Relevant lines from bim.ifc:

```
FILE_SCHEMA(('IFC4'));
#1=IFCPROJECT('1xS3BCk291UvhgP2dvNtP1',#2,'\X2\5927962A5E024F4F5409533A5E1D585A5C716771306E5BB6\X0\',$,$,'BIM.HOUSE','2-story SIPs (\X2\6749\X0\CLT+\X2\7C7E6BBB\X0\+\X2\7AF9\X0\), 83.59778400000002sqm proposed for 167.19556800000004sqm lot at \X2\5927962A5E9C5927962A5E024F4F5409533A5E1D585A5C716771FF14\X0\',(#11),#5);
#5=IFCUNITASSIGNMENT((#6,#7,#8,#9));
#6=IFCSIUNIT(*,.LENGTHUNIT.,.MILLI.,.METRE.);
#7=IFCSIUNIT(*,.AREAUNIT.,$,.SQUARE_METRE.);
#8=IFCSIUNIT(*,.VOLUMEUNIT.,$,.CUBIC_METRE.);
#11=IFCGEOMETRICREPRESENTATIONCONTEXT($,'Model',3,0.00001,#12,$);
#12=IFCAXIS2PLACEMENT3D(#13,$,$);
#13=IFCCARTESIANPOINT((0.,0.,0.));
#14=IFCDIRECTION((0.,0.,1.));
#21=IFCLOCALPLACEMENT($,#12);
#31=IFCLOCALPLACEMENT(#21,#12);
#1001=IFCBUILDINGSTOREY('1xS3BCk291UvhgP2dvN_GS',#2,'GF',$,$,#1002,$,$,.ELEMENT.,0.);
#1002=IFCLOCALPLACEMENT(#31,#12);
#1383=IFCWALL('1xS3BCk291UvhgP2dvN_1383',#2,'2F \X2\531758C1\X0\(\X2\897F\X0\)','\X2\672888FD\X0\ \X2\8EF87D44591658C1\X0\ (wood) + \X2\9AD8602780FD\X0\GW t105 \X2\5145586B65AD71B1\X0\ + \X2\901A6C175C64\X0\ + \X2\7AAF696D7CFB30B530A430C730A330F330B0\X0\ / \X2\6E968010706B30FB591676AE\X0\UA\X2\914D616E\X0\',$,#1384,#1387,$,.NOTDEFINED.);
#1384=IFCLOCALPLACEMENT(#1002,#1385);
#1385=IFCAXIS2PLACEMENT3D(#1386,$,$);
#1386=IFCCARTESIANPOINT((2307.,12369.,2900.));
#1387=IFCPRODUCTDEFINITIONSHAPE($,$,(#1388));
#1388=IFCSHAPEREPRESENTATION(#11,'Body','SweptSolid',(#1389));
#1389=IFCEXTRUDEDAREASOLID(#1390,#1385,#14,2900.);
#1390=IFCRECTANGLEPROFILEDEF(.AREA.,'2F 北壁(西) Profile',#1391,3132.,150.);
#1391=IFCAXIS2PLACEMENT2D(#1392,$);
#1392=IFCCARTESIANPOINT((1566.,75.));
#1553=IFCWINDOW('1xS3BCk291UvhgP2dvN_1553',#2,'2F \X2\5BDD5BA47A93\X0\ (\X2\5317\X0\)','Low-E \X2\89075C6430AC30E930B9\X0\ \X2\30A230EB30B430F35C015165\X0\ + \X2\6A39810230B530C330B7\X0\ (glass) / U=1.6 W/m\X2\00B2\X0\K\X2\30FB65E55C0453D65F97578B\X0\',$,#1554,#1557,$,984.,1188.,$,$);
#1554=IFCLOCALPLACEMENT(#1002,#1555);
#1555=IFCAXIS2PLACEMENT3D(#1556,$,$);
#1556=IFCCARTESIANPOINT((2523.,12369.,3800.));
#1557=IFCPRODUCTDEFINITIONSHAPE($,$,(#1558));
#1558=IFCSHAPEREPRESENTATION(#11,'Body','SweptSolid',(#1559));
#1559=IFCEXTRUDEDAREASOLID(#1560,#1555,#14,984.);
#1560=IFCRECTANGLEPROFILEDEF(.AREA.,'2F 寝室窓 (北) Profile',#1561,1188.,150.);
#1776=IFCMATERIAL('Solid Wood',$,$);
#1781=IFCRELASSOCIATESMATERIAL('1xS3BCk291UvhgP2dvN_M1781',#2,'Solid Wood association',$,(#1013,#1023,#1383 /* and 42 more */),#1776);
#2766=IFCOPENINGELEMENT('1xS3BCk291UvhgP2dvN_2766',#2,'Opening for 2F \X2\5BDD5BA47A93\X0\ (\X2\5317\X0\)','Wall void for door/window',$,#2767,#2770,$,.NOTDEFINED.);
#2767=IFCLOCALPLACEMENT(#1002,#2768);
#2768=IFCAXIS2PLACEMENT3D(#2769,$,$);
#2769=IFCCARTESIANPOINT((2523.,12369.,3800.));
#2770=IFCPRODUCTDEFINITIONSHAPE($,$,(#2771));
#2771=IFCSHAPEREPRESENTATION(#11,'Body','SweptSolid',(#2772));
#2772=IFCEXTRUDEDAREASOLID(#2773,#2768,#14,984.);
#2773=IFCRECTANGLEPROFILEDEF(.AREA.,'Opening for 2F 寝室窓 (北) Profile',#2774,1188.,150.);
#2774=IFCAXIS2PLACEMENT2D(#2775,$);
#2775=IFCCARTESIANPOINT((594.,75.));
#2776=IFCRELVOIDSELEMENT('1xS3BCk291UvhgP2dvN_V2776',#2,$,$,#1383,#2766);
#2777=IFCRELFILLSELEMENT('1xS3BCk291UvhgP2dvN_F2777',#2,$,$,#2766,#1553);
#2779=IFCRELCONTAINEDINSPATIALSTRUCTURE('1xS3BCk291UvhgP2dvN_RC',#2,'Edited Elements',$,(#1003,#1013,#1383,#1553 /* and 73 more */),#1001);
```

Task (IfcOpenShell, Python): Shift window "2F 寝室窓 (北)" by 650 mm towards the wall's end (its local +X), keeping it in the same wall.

```python
import ifcopenshell
import ifcopenshell.api.geometry
import ifcopenshell.util.placement

model = ifcopenshell.open("bim.ifc")

window = model.by_id(1553)
opening = window.FillsVoids[0].RelatingOpeningElement
wall = opening.VoidsElements[0].RelatingBuildingElement

wall_matrix = ifcopenshell.util.placement.get_local_placement(wall.ObjectPlacement)
shift = wall_matrix[:3, 0] * 650.0
before = ifcopenshell.util.placement.get_local_placement(window.ObjectPlacement)[:3, 3].copy()

# The window is not placed relative to its opening, so move both.
for product in (opening, window):
    matrix = ifcopenshell.util.placement.get_local_placement(product.ObjectPlacement)
    matrix[:3, 3] += shift
    ifcopenshell.api.geometry.edit_object_placement(model, product=product, matrix=matrix, is_si=False)

after = ifcopenshell.util.placement.get_local_placement(window.ObjectPlacement)[:3, 3]
print("window moved by", (after - before).round(3) + 0.0)

model.write("bim_rev.ifc")
```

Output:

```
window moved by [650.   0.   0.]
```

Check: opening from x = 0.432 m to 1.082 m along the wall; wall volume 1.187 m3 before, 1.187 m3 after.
